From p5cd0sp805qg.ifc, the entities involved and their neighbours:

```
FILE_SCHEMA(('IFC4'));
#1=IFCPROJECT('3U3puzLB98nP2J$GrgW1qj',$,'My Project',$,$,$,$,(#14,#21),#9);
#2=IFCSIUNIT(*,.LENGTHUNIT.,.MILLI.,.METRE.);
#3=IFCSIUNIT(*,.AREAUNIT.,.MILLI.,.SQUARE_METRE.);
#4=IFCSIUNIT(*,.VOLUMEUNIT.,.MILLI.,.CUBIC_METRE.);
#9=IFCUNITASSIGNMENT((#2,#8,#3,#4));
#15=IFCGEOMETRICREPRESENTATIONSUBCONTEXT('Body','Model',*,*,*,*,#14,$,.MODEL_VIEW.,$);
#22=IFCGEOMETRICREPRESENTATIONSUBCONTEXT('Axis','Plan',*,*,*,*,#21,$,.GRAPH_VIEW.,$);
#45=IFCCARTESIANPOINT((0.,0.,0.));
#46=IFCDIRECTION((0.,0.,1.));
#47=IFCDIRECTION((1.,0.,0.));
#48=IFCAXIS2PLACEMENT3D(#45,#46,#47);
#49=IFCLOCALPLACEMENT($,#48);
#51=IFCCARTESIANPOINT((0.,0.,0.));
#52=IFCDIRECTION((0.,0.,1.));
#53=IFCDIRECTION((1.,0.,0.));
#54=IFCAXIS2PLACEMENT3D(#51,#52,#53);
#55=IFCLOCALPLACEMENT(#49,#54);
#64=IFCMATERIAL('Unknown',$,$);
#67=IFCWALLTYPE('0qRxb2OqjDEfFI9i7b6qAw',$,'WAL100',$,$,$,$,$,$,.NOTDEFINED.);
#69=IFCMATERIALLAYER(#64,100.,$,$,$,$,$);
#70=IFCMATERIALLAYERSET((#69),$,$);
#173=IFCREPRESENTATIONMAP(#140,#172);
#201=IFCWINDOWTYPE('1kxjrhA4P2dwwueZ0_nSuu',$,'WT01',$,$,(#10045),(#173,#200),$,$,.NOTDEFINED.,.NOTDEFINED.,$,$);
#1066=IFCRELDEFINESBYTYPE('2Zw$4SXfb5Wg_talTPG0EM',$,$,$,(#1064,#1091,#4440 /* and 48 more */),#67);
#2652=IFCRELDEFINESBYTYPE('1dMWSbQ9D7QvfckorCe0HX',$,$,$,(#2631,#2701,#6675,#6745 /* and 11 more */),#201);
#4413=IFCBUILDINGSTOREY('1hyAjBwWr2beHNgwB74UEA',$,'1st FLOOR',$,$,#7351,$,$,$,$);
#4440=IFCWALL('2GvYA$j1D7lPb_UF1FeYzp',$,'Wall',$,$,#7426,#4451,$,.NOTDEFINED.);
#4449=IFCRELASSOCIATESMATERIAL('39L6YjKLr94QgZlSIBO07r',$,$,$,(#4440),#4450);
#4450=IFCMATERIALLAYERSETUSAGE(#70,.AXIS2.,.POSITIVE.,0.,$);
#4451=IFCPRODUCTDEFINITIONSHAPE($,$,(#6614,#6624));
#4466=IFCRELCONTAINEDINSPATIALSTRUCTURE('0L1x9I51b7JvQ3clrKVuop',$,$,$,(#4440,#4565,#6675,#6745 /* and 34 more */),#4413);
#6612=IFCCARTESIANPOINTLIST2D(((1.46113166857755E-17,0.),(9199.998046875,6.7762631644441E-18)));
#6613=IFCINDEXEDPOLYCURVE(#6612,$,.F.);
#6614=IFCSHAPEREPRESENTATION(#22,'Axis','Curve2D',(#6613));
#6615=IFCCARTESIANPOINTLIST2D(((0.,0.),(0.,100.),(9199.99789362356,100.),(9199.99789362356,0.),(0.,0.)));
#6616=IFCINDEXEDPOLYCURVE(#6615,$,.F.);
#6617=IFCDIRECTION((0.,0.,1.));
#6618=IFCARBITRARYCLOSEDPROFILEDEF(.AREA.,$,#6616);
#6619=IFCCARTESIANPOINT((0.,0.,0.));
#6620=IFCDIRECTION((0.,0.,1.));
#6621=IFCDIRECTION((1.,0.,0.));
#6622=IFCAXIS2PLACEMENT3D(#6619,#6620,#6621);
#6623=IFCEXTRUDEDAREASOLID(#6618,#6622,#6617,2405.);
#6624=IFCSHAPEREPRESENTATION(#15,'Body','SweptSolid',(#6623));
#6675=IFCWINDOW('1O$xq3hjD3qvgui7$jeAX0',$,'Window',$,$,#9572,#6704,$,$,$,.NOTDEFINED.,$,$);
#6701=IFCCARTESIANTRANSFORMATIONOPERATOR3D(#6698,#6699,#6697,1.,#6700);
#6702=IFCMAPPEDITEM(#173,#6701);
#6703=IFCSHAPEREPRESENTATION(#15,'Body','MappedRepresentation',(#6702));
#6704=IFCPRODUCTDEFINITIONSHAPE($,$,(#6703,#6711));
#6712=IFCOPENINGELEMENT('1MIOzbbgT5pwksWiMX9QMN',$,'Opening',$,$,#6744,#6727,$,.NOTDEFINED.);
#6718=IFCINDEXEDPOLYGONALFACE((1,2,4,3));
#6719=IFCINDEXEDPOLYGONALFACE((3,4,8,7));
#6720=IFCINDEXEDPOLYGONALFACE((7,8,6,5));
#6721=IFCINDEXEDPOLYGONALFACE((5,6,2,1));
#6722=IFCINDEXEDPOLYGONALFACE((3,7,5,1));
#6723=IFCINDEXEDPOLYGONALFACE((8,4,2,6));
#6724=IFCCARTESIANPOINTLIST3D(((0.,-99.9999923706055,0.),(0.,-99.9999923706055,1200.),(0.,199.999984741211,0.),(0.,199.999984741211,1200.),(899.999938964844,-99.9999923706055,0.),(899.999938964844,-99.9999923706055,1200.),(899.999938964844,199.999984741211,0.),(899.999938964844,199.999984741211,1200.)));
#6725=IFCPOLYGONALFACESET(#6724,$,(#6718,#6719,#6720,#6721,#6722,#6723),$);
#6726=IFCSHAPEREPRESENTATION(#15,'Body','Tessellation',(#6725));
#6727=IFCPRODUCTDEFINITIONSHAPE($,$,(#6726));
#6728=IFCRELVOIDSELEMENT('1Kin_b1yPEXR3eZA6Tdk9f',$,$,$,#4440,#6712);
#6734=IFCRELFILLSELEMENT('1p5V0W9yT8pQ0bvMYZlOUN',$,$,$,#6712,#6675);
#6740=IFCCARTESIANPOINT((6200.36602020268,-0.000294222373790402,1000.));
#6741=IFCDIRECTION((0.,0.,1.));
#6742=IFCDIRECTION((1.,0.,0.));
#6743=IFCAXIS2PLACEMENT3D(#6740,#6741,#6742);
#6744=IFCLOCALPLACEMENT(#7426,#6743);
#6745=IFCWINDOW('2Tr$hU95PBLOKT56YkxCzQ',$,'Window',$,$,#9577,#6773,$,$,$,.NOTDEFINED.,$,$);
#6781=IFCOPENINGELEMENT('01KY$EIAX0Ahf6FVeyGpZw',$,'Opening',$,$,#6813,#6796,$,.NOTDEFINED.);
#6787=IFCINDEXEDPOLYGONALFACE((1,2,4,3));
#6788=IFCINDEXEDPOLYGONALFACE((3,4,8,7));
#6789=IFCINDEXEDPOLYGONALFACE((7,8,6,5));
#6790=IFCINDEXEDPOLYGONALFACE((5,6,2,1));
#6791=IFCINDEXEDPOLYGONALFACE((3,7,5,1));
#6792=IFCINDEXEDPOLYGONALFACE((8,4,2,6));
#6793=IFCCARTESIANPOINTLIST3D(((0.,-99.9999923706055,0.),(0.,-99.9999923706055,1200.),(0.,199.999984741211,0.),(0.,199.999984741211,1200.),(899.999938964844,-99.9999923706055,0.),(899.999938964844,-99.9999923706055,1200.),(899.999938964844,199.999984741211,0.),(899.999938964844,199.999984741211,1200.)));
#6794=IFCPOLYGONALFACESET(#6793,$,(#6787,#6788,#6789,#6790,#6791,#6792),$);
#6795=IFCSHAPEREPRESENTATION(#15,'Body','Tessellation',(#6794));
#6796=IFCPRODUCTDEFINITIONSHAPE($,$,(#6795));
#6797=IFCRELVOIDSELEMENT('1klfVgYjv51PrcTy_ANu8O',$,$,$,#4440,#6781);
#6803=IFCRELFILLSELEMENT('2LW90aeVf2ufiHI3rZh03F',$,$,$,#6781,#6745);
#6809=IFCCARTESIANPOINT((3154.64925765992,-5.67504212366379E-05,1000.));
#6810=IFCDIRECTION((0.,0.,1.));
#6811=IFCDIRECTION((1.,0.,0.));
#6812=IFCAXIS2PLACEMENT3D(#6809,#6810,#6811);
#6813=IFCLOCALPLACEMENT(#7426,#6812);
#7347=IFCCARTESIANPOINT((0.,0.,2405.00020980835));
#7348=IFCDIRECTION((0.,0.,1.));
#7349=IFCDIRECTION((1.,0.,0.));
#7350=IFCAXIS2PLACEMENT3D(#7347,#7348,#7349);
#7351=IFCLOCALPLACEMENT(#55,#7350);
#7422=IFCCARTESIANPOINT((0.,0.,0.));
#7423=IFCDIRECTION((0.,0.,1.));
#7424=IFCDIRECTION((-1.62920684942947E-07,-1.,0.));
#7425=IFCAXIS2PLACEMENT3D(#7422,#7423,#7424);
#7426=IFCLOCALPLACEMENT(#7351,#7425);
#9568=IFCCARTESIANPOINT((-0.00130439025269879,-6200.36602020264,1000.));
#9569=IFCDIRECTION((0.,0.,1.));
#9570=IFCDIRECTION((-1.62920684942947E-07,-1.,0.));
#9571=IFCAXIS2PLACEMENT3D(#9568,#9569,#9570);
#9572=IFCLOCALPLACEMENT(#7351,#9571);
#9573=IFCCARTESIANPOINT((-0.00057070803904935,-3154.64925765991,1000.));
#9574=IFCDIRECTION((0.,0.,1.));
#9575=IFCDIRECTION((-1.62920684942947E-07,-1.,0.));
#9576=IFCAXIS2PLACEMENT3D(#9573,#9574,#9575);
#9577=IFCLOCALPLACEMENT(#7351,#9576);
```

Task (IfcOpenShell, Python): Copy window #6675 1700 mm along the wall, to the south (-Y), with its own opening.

```python
import ifcopenshell
import ifcopenshell.api.feature
import ifcopenshell.api.geometry
import ifcopenshell.api.root
import ifcopenshell.geom
import ifcopenshell.util.element
import ifcopenshell.util.placement
import ifcopenshell.util.shape

model = ifcopenshell.open("p5cd0sp805qg.ifc")
settings = ifcopenshell.geom.settings()


def volume(element):
    """Net volume in cubic metres, openings subtracted."""
    shape = ifcopenshell.geom.create_shape(settings, element)
    return ifcopenshell.util.shape.get_volume(shape.geometry)


window = model.by_guid("1O$xq3hjD3qvgui7$jeAX0")
opening = window.FillsVoids[0].RelatingOpeningElement
wall = opening.VoidsElements[0].RelatingBuildingElement
before = volume(wall)
shift = ifcopenshell.util.placement.get_local_placement(wall.ObjectPlacement)[:3, 0] * 1700.0

# copy_class copies the void relationship, type, container and properties, but no geometry.
new_opening = ifcopenshell.api.root.copy_class(model, product=opening)
new_opening.Representation = ifcopenshell.util.element.copy_deep(
    model, opening.Representation, exclude=["IfcGeometricRepresentationContext", "IfcRepresentationMap"]
)
new_window = ifcopenshell.api.root.copy_class(model, product=window)
new_window.Representation = ifcopenshell.util.element.copy_deep(
    model, window.Representation, exclude=["IfcGeometricRepresentationContext", "IfcRepresentationMap"]
)
ifcopenshell.api.feature.add_filling(model, opening=new_opening, element=new_window)

for old, new in ((opening, new_opening), (window, new_window)):
    matrix = ifcopenshell.util.placement.get_local_placement(old.ObjectPlacement)
    matrix[:3, 3] += shift
    ifcopenshell.api.geometry.edit_object_placement(model, product=new, matrix=matrix, is_si=False)

after = volume(wall)

print(f"wall volume {before:.3f} -> {after:.3f} m3")

model.write("p5cd0sp805qg_rev.ifc")
```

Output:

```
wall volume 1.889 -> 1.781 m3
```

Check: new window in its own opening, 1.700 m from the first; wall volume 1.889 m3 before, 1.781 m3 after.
